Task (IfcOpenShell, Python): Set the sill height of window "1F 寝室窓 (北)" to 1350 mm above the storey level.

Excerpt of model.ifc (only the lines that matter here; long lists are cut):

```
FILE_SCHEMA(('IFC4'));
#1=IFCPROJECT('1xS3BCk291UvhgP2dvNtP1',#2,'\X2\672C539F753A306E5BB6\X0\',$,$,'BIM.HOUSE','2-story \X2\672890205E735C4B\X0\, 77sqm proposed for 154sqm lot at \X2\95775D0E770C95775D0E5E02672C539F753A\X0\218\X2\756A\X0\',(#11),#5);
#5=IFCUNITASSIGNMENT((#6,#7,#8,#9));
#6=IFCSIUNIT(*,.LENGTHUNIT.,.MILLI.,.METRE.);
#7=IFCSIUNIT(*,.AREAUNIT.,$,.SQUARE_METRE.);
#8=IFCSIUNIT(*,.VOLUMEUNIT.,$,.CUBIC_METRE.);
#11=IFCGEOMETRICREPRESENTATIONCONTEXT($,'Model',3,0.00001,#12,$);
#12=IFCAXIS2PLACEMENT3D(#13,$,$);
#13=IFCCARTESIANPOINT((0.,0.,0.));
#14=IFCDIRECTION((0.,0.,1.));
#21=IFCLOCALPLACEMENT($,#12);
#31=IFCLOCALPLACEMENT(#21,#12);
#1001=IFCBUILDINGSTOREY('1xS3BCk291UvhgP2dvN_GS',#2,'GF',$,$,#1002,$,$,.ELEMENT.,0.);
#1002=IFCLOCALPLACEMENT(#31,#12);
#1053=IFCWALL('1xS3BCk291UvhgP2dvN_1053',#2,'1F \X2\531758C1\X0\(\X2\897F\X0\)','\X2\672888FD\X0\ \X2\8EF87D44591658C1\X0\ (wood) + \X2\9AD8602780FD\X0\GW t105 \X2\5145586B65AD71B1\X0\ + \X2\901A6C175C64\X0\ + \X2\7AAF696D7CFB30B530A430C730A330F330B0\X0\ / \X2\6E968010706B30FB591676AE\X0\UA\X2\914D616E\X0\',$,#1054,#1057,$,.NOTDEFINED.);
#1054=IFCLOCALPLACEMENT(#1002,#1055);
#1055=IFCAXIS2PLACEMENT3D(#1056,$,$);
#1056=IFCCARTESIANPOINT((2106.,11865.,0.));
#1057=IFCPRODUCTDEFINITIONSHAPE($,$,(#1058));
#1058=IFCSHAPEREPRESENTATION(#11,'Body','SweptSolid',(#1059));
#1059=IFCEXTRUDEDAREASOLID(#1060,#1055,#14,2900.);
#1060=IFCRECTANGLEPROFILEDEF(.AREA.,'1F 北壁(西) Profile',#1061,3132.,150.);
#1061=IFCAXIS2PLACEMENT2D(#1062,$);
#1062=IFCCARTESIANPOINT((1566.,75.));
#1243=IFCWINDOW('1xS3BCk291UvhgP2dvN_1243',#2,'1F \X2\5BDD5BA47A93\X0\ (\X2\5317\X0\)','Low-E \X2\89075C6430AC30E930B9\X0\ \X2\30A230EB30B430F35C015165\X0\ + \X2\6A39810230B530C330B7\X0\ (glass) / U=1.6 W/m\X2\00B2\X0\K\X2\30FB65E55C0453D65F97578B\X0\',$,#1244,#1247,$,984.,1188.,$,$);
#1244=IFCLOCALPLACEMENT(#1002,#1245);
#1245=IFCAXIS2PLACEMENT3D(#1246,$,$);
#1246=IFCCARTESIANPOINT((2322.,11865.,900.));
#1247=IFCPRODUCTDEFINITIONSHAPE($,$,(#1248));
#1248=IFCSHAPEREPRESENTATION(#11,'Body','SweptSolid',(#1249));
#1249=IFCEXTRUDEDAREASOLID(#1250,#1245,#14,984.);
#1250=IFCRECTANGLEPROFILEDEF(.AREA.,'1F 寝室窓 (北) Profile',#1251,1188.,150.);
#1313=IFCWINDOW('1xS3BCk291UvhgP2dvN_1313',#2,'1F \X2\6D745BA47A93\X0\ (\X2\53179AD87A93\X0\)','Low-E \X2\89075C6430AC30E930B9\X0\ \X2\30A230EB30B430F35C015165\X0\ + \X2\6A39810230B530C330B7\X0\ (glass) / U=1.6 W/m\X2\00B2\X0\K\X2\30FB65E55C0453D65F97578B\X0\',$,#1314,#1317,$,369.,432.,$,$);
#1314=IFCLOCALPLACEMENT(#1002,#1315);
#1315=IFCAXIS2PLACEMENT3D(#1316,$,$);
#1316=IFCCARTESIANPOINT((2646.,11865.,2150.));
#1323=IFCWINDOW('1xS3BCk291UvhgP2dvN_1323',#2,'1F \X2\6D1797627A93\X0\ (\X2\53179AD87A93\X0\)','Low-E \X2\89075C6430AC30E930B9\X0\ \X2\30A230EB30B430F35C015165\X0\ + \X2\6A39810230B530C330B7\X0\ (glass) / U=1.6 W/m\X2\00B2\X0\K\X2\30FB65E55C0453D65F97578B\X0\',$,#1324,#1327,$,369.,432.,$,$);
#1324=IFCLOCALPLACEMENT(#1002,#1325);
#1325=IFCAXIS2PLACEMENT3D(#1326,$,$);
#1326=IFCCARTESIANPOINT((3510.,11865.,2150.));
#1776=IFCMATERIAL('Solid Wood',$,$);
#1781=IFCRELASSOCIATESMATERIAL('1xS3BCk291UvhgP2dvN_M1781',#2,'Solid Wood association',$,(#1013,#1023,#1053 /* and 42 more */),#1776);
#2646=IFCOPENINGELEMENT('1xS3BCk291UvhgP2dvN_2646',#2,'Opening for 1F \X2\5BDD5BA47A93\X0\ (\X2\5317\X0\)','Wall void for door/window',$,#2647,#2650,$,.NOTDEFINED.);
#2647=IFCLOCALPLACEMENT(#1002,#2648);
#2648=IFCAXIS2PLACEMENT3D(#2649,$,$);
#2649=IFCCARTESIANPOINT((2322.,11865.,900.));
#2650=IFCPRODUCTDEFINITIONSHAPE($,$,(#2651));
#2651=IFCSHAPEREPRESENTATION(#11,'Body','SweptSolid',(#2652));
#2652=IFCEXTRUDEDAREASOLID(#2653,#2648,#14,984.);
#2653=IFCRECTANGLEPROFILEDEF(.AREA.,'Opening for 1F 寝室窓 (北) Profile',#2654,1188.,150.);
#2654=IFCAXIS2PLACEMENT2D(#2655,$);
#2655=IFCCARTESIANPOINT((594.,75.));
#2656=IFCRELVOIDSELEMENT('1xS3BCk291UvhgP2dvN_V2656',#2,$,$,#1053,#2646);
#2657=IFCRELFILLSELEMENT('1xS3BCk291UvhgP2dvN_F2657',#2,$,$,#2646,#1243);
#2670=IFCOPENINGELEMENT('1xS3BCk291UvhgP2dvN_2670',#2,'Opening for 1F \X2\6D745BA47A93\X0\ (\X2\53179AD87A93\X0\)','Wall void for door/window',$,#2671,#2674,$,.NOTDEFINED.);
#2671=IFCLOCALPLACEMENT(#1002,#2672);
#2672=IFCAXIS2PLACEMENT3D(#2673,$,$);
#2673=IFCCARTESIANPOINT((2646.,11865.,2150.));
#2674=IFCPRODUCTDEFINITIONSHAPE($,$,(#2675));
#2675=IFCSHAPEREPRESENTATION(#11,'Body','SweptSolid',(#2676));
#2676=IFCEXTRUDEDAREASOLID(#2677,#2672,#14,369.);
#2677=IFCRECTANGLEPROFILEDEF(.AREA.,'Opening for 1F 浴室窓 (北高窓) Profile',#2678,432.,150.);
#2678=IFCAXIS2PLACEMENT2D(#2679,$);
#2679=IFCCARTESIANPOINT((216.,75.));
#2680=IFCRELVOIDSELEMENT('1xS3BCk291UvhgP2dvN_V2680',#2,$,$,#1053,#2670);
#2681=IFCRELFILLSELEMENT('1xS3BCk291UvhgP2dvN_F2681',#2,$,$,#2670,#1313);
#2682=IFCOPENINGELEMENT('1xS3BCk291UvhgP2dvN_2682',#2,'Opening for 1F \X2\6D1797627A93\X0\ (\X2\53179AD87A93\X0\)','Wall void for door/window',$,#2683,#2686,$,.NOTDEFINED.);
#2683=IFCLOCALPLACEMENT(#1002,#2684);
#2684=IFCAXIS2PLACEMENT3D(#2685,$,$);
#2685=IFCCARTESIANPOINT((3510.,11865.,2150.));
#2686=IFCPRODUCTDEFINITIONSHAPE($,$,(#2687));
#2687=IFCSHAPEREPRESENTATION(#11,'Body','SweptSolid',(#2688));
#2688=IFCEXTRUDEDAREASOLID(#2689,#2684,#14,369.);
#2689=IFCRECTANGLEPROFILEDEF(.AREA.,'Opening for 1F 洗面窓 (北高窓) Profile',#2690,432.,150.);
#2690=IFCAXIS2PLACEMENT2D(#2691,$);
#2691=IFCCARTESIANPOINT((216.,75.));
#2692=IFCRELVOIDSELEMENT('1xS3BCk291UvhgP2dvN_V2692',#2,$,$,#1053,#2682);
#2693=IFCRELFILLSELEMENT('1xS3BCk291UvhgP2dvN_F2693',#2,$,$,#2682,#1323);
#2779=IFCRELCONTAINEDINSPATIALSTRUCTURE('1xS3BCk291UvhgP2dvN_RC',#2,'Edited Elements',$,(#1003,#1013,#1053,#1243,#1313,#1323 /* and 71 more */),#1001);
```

```python
import numpy as np
import ifcopenshell
import ifcopenshell.api.geometry
import ifcopenshell.geom
import ifcopenshell.util.element
import ifcopenshell.util.placement
import ifcopenshell.util.shape
import ifcopenshell.util.unit

model = ifcopenshell.open("model.ifc")
unit_scale = ifcopenshell.util.unit.calculate_unit_scale(model)

window = model.by_guid("1xS3BCk291UvhgP2dvN_1243")
opening = window.FillsVoids[0].RelatingOpeningElement
storey = ifcopenshell.util.element.get_container(window, ifc_class="IfcBuildingStorey")
level = ifcopenshell.util.placement.get_local_placement(storey.ObjectPlacement)[2, 3]

# The opening's origin need not be at the sill, so measure its lowest point.
shape = ifcopenshell.geom.create_shape(ifcopenshell.geom.settings(), opening)
bottom = ifcopenshell.util.shape.get_shape_bottom_elevation(shape, shape.geometry) / unit_scale
dz = level + 1.35 / unit_scale - bottom

shift = np.array([0.0, 0.0, dz])
# The window is not placed relative to its opening, so move both.
for product in (opening, window):
    matrix = ifcopenshell.util.placement.get_local_placement(product.ObjectPlacement)
    matrix[:3, 3] += shift
    ifcopenshell.api.geometry.edit_object_placement(model, product=product, matrix=matrix, is_si=False)

print(f"moved by {dz * unit_scale:+.3f} m")

model.write("model_rev.ifc")
```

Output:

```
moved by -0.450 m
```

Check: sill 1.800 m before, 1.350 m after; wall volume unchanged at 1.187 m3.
